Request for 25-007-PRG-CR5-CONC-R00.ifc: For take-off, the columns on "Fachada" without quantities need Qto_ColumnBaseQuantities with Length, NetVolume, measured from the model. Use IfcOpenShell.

First a look at what the model holds.

```python
import ifcopenshell
import ifcopenshell.util.element
import ifcopenshell.util.unit

model = ifcopenshell.open("25-007-PRG-CR5-CONC-R00.ifc")
print(model.schema)
for unit_type in ("LENGTHUNIT", "AREAUNIT", "VOLUMEUNIT"):
    print(unit_type, ifcopenshell.util.unit.calculate_unit_scale(model, unit_type))
storey = next(s for s in model.by_type("IfcBuildingStorey") if s.Name == "Fachada")
columns = [e for e in ifcopenshell.util.element.get_decomposition(storey) if e.is_a("IfcColumn")]
for e in sorted(columns, key=lambda e: e.id()):
    print(e.id(), e.is_a(), e.Name, list(ifcopenshell.util.element.get_psets(e, qtos_only=True)), sep=" | ")
```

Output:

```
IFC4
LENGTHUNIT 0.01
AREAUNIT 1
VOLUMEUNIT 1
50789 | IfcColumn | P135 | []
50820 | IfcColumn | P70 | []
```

```python
import ifcopenshell
import ifcopenshell.api.pset
import ifcopenshell.geom
import ifcopenshell.util.element
import ifcopenshell.util.shape
import ifcopenshell.util.unit

model = ifcopenshell.open("25-007-PRG-CR5-CONC-R00.ifc")
unit_scale = ifcopenshell.util.unit.calculate_unit_scale(model)
volume_scale = ifcopenshell.util.unit.calculate_unit_scale(model, "VOLUMEUNIT")
settings = ifcopenshell.geom.settings()

storey = next(s for s in model.by_type("IfcBuildingStorey") if s.Name == "Fachada")
columns = [e for e in ifcopenshell.util.element.get_decomposition(storey) if e.is_a("IfcColumn")]

for e in sorted(columns, key=lambda e: e.id()):
    if ifcopenshell.util.element.get_psets(e, qtos_only=True, should_inherit=False):
        continue
    # Geometry comes back in metres, in the element's own axes.
    shape = ifcopenshell.geom.create_shape(settings, e)
    values = {
        "Length": ifcopenshell.util.shape.get_z(shape.geometry) / unit_scale,
        "NetVolume": ifcopenshell.util.shape.get_volume(shape.geometry) / volume_scale,
    }
    qto = ifcopenshell.api.pset.add_qto(model, product=e, name="Qto_ColumnBaseQuantities")
    ifcopenshell.api.pset.edit_qto(model, qto=qto, properties=values)
    print(e.id(), {k: round(v, 3) for k, v in values.items()})

model.write("25-007-PRG-CR5-CONC-R00_updated.ifc")
```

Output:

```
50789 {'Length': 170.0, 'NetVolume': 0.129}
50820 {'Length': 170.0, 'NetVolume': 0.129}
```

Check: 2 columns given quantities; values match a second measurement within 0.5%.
